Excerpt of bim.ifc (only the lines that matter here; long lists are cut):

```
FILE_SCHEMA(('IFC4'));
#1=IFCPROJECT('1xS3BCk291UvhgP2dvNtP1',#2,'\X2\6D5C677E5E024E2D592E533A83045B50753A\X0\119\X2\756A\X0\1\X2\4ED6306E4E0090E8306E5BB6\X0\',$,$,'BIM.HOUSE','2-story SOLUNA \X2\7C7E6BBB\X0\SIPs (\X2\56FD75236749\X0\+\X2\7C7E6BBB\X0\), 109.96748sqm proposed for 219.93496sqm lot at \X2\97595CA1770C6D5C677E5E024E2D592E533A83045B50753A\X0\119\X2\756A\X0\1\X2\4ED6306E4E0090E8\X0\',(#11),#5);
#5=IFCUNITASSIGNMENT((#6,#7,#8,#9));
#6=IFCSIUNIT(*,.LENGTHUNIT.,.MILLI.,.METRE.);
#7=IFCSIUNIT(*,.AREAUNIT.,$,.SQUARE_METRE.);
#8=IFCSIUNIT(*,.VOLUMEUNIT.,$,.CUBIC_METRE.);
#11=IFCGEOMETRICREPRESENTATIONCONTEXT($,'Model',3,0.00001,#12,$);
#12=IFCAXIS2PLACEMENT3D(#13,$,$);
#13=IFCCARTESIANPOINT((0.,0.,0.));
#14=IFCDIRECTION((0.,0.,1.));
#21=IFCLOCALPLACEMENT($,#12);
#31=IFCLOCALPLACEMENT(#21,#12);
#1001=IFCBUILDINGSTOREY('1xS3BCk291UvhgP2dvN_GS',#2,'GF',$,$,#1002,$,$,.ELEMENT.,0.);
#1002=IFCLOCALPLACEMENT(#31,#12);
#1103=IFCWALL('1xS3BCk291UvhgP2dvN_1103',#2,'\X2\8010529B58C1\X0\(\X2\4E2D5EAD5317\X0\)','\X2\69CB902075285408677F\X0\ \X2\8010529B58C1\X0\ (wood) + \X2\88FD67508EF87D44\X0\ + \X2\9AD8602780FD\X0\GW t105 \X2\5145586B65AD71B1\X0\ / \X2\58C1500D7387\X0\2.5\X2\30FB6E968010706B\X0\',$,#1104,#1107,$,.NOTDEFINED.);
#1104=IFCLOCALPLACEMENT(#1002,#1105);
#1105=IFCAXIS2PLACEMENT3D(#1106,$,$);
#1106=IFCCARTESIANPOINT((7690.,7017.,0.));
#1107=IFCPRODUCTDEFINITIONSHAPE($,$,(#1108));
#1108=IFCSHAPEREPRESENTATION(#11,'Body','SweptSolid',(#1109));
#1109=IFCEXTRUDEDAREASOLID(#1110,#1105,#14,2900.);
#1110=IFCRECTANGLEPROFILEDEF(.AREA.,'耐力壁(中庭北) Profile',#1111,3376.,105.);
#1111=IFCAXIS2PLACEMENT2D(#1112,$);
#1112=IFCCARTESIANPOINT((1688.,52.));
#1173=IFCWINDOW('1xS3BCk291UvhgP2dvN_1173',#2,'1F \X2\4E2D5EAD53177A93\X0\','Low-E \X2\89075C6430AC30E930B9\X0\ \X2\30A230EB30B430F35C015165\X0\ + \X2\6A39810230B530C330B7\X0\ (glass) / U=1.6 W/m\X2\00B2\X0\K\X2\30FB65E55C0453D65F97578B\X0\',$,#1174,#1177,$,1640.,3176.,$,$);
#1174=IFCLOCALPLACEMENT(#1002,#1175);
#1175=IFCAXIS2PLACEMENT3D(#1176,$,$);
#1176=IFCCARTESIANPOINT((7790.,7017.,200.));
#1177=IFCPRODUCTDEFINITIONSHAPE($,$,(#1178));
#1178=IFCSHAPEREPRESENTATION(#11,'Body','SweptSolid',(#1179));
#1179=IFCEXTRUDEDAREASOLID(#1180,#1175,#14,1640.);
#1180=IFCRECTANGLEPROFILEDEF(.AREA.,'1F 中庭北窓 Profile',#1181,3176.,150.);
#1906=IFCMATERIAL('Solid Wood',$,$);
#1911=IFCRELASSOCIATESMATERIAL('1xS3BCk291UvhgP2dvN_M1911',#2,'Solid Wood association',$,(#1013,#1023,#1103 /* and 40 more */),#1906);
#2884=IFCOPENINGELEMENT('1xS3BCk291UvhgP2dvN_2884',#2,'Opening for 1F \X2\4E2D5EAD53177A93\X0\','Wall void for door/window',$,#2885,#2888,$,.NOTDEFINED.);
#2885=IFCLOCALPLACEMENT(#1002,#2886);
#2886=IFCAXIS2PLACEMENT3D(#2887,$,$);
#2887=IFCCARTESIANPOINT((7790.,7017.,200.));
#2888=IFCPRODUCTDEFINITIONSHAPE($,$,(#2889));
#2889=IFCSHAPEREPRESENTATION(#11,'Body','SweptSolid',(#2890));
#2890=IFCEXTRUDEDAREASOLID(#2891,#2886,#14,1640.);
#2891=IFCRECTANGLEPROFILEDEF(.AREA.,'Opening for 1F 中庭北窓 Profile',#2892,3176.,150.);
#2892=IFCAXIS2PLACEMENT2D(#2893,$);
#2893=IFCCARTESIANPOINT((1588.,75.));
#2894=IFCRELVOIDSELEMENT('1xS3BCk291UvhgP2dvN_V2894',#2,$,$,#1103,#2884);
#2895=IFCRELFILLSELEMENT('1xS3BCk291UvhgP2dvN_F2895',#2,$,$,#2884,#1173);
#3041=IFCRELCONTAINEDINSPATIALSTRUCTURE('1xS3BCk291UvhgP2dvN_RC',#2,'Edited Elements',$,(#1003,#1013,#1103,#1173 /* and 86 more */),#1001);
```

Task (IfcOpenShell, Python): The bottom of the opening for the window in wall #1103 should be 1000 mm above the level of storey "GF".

```python
import numpy as np
import ifcopenshell
import ifcopenshell.api.geometry
import ifcopenshell.geom
import ifcopenshell.util.element
import ifcopenshell.util.placement
import ifcopenshell.util.shape
import ifcopenshell.util.unit

model = ifcopenshell.open("bim.ifc")
unit_scale = ifcopenshell.util.unit.calculate_unit_scale(model)

window = model.by_guid("1xS3BCk291UvhgP2dvN_1173")
opening = window.FillsVoids[0].RelatingOpeningElement
storey = ifcopenshell.util.element.get_container(window, ifc_class="IfcBuildingStorey")
level = ifcopenshell.util.placement.get_local_placement(storey.ObjectPlacement)[2, 3]

# The opening's origin need not be at the sill, so measure its lowest point.
shape = ifcopenshell.geom.create_shape(ifcopenshell.geom.settings(), opening)
bottom = ifcopenshell.util.shape.get_shape_bottom_elevation(shape, shape.geometry) / unit_scale
dz = level + 1 / unit_scale - bottom

shift = np.array([0.0, 0.0, dz])
# The window is not placed relative to its opening, so move both.
for product in (opening, window):
    matrix = ifcopenshell.util.placement.get_local_placement(product.ObjectPlacement)
    matrix[:3, 3] += shift
    ifcopenshell.api.geometry.edit_object_placement(model, product=product, matrix=matrix, is_si=False)

print(f"moved by {dz * unit_scale:+.3f} m")

model.write("bim_rev.ifc")
```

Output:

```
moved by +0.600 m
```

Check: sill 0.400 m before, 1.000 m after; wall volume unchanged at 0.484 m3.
